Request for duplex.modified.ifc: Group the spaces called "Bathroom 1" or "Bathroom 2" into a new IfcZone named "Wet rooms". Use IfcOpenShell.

First a look at what the model holds.

```python
import ifcopenshell

model = ifcopenshell.open("duplex.modified.ifc")
print(model.schema)
seen = {}
for space in model.by_type("IfcSpace"):
    seen[space.LongName] = seen.get(space.LongName, 0) + 1
for name, count in sorted(seen.items(), key=str):
    print(count, "x", name)
print("zones:", [z.Name for z in model.by_type("IfcZone")][:20])
```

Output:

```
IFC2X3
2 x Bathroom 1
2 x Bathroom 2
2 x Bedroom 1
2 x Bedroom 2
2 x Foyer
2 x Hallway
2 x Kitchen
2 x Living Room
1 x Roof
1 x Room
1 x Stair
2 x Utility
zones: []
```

```python
import ifcopenshell
import ifcopenshell.api.group
import ifcopenshell.api.root

model = ifcopenshell.open("duplex.modified.ifc")

names = {"Bathroom 1", "Bathroom 2"}
spaces = [s for s in model.by_type("IfcSpace") if s.LongName in names]

zone = ifcopenshell.api.root.create_entity(model, ifc_class="IfcZone", name="Wet rooms")
ifcopenshell.api.group.assign_group(model, products=spaces, group=zone)
print(len(spaces), "spaces in", zone.Name)

model.write("duplex.modified_rev.ifc")
```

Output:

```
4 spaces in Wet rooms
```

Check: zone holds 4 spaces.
